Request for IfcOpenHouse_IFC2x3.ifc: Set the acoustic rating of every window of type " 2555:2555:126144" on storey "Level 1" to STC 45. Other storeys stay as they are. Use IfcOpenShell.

First a look at what the model holds.

```python
import ifcopenshell
import ifcopenshell.util.element

model = ifcopenshell.open("IfcOpenHouse_IFC2x3.ifc")
print(model.schema)
storey = next(s for s in model.by_type("IfcBuildingStorey") if s.Name == "Level 1")
windows = [e for e in ifcopenshell.util.element.get_decomposition(storey) if e.is_a("IfcWindow")]
seen = {}
for e in windows:
    element_type = ifcopenshell.util.element.get_type(e)
    key = (element_type.Name if element_type != e and element_type else None, ifcopenshell.util.element.get_pset(e, "Pset_WindowCommon", "AcousticRating"))
    seen[key] = seen.get(key, 0) + 1
for (name, value), count in sorted(seen.items(), key=str):
    print(count, "x", name, "|", value)
```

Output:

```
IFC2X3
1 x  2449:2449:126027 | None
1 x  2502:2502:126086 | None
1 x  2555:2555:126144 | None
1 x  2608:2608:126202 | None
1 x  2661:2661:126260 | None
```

```python
import ifcopenshell
import ifcopenshell.api.pset
import ifcopenshell.util.element

model = ifcopenshell.open("IfcOpenHouse_IFC2x3.ifc")

storey = next(s for s in model.by_type("IfcBuildingStorey") if s.Name == "Level 1")
windows = [e for e in ifcopenshell.util.element.get_decomposition(storey) if e.is_a("IfcWindow")]

count = 0
for e in windows:
    element_type = ifcopenshell.util.element.get_type(e)
    if element_type in (None, e) or element_type.Name != " 2555:2555:126144":
        continue
    # add_pset returns the element's existing set when there is one.
    pset = ifcopenshell.api.pset.add_pset(model, product=e, name="Pset_WindowCommon")
    ifcopenshell.api.pset.edit_pset(model, pset=pset, properties={"AcousticRating": "STC 45"})
    count += 1

print(count, "windows updated")

model.write("IfcOpenHouse_IFC2x3_updated.ifc")
```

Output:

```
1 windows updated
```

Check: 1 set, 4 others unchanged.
